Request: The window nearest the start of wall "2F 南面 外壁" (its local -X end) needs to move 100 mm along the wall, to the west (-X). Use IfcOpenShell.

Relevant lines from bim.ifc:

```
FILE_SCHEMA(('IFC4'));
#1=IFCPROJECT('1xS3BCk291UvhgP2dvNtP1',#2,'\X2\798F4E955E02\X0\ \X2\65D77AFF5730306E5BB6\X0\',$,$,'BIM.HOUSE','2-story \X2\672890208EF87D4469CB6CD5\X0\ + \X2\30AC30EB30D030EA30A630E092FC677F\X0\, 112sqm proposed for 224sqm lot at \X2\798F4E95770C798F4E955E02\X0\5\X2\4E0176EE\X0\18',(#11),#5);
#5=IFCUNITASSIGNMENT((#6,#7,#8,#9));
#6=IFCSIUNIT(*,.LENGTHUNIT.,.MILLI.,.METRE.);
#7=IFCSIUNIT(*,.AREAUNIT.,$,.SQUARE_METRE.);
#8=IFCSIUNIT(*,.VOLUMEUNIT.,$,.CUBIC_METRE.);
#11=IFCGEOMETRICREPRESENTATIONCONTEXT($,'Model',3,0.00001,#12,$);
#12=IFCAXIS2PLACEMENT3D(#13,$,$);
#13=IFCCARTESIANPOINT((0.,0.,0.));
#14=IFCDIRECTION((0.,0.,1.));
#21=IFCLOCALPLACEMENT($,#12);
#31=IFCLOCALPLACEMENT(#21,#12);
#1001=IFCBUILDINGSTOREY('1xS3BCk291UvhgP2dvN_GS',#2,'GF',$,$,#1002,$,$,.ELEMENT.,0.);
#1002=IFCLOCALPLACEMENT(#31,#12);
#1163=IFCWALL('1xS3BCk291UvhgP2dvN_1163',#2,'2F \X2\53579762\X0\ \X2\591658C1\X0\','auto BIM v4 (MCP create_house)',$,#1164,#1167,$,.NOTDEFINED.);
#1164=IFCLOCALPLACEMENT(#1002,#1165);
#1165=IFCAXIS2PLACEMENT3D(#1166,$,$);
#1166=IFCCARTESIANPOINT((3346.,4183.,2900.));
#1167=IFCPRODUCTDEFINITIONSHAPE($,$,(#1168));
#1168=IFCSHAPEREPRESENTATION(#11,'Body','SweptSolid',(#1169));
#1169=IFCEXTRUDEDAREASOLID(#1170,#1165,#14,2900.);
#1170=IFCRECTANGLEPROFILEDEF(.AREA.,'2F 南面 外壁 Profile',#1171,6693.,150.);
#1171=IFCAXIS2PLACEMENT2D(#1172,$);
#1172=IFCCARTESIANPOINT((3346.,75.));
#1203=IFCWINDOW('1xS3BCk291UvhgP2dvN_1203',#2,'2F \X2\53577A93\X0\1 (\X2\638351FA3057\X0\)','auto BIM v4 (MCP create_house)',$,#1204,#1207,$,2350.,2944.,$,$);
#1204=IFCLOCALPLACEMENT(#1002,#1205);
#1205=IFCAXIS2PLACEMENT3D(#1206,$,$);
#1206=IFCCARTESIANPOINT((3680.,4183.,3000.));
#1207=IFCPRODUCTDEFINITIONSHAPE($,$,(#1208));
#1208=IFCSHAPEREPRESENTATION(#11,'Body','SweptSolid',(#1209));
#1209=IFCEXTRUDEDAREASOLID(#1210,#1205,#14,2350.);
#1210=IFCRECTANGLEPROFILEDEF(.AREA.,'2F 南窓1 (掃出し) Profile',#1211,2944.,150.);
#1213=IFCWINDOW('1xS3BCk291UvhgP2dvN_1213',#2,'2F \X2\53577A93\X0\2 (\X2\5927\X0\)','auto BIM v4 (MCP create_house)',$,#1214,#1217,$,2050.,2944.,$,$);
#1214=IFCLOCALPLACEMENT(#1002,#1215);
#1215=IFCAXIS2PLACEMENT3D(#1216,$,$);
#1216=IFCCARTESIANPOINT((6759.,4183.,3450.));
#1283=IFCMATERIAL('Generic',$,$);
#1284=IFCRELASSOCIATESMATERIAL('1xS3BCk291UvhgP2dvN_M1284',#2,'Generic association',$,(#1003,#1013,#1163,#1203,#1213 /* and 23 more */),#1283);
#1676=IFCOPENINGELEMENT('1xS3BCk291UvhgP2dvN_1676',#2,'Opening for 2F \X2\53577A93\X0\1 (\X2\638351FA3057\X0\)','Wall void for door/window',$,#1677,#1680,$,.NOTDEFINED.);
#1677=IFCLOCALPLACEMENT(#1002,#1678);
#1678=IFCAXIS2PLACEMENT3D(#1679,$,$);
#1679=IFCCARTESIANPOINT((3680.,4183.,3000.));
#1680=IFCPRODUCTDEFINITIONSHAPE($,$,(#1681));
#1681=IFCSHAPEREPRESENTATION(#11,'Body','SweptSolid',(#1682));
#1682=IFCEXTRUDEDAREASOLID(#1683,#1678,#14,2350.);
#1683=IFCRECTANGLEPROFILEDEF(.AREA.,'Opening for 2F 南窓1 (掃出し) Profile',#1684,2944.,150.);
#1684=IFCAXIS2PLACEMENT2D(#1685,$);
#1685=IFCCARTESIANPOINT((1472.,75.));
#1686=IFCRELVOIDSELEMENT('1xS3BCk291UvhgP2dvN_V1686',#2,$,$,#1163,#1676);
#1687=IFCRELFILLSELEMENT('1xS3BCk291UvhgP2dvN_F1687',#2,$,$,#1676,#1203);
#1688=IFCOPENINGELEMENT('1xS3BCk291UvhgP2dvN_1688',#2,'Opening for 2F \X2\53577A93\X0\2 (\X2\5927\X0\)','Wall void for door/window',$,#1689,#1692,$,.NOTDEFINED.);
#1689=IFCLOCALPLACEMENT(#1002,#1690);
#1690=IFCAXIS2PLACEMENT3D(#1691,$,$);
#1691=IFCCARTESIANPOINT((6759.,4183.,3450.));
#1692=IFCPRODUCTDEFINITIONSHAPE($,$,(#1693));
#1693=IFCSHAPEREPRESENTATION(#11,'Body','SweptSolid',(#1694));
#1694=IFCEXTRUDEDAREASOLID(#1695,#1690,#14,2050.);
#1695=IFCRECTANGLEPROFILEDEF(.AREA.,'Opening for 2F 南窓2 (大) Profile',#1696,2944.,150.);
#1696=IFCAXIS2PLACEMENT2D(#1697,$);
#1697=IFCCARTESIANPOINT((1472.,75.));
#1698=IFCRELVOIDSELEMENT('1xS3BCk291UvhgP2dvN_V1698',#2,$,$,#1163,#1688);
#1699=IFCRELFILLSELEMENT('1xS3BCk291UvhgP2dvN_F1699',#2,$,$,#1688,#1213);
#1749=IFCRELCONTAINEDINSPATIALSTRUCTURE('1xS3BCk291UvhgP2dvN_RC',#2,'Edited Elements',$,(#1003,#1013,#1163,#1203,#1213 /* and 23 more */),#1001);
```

```python
import ifcopenshell
import ifcopenshell.api.geometry
import ifcopenshell.util.placement
import ifcopenshell.util.unit

model = ifcopenshell.open("bim.ifc")
unit_scale = ifcopenshell.util.unit.calculate_unit_scale(model)

window = model.by_guid("1xS3BCk291UvhgP2dvN_1203")
opening = window.FillsVoids[0].RelatingOpeningElement
wall = opening.VoidsElements[0].RelatingBuildingElement

wall_matrix = ifcopenshell.util.placement.get_local_placement(wall.ObjectPlacement)
shift = wall_matrix[:3, 0] * -0.1 / unit_scale
before = ifcopenshell.util.placement.get_local_placement(window.ObjectPlacement)[:3, 3].copy()

# The window is not placed relative to its opening, so move both.
for product in (opening, window):
    matrix = ifcopenshell.util.placement.get_local_placement(product.ObjectPlacement)
    matrix[:3, 3] += shift
    ifcopenshell.api.geometry.edit_object_placement(model, product=product, matrix=matrix, is_si=False)

after = ifcopenshell.util.placement.get_local_placement(window.ObjectPlacement)[:3, 3]
print("window moved by", (after - before).round(3) + 0.0)

model.write("bim_v2.ifc")
```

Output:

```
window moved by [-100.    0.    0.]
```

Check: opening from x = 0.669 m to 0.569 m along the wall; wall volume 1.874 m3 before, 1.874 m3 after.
